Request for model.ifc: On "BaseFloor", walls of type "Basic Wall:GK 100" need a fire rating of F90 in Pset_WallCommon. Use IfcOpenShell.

First a look at what the model holds.

```python
import ifcopenshell
import ifcopenshell.util.element

model = ifcopenshell.open("model.ifc")
print(model.schema)
storey = next(s for s in model.by_type("IfcBuildingStorey") if s.Name == "BaseFloor")
walls = [e for e in ifcopenshell.util.element.get_decomposition(storey) if e.is_a("IfcWall")]
seen = {}
for e in walls:
    element_type = ifcopenshell.util.element.get_type(e)
    key = (element_type.Name if element_type != e and element_type else None, ifcopenshell.util.element.get_pset(e, "Pset_WallCommon", "FireRating"))
    seen[key] = seen.get(key, 0) + 1
for (name, value), count in sorted(seen.items(), key=str):
    print(count, "x", name, "|", value)
```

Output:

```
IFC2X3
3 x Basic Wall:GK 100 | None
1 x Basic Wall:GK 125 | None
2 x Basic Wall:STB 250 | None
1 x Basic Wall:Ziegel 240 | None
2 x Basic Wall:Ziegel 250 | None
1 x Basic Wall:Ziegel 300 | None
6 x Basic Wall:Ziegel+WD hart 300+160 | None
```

```python
import ifcopenshell
import ifcopenshell.api.pset
import ifcopenshell.util.element

model = ifcopenshell.open("model.ifc")

storey = next(s for s in model.by_type("IfcBuildingStorey") if s.Name == "BaseFloor")
walls = [e for e in ifcopenshell.util.element.get_decomposition(storey) if e.is_a("IfcWall")]

count = 0
for e in walls:
    element_type = ifcopenshell.util.element.get_type(e)
    if element_type in (None, e) or element_type.Name != "Basic Wall:GK 100":
        continue
    # add_pset returns the element's existing set when there is one.
    pset = ifcopenshell.api.pset.add_pset(model, product=e, name="Pset_WallCommon")
    ifcopenshell.api.pset.edit_pset(model, pset=pset, properties={"FireRating": "F90"})
    count += 1

print(count, "walls updated")

model.write("model_rev.ifc")
```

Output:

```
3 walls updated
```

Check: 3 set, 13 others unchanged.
